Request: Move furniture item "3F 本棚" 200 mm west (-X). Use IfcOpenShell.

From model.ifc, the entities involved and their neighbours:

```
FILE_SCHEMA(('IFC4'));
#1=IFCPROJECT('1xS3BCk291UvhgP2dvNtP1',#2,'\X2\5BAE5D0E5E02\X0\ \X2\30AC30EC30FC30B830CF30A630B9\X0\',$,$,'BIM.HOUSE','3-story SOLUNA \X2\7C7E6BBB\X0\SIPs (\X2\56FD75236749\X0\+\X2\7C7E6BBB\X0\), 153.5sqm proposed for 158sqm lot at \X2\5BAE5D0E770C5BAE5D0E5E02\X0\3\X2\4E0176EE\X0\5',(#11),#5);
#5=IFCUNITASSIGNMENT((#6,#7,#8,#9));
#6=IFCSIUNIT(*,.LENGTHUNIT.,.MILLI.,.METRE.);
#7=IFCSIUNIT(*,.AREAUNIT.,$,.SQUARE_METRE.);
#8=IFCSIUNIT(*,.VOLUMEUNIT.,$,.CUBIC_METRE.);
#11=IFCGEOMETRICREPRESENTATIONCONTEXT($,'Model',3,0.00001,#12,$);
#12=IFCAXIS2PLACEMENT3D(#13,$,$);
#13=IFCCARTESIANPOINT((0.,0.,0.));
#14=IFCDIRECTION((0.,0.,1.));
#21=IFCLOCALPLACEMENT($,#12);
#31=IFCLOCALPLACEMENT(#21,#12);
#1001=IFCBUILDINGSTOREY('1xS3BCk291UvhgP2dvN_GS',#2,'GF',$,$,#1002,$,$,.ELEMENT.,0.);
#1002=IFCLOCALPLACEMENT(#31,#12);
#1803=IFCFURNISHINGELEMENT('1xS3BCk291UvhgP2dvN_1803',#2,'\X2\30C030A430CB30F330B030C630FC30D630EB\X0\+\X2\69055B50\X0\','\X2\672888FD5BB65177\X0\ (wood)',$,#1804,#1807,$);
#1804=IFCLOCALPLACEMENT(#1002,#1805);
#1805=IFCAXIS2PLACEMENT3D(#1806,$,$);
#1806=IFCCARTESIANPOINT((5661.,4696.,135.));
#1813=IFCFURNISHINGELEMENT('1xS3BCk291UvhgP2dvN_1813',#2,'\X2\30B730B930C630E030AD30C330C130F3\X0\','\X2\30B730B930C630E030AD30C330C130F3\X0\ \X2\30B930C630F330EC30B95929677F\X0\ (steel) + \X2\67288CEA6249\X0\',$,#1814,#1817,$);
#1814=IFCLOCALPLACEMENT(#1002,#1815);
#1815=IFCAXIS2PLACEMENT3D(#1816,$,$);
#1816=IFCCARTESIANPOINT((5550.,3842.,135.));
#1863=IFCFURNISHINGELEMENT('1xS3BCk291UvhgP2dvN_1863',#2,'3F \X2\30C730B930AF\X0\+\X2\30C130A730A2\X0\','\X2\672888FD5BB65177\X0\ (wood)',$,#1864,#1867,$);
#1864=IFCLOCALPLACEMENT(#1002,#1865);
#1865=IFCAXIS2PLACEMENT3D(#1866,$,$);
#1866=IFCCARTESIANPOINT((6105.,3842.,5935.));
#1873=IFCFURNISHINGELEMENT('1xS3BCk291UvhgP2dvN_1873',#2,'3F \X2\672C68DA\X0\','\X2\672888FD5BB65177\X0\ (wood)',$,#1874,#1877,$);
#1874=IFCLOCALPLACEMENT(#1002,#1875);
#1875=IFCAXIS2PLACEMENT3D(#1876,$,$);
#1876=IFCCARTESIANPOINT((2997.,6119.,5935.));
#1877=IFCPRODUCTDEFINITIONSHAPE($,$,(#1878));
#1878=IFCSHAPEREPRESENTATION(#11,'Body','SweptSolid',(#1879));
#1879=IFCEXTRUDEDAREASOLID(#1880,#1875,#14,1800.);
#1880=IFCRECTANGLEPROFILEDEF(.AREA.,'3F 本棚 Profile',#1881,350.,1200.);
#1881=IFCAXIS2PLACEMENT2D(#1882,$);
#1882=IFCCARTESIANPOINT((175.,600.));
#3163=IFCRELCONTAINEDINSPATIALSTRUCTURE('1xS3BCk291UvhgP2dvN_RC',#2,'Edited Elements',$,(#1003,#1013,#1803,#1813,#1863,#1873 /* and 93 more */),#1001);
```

```python
import ifcopenshell
import ifcopenshell.api.geometry
import ifcopenshell.util.placement

model = ifcopenshell.open("model.ifc")

item = model.by_guid("1xS3BCk291UvhgP2dvN_1873")
matrix = ifcopenshell.util.placement.get_local_placement(item.ObjectPlacement)
matrix[0, 3] -= 200.0
ifcopenshell.api.geometry.edit_object_placement(model, product=item, matrix=matrix, is_si=False)

print(ifcopenshell.util.placement.get_local_placement(item.ObjectPlacement).round(3) + 0.0)

model.write("model_edited.ifc")
```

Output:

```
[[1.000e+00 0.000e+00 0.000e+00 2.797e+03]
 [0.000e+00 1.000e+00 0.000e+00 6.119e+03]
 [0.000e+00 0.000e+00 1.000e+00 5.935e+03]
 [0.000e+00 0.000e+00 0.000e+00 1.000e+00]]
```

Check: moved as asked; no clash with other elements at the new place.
